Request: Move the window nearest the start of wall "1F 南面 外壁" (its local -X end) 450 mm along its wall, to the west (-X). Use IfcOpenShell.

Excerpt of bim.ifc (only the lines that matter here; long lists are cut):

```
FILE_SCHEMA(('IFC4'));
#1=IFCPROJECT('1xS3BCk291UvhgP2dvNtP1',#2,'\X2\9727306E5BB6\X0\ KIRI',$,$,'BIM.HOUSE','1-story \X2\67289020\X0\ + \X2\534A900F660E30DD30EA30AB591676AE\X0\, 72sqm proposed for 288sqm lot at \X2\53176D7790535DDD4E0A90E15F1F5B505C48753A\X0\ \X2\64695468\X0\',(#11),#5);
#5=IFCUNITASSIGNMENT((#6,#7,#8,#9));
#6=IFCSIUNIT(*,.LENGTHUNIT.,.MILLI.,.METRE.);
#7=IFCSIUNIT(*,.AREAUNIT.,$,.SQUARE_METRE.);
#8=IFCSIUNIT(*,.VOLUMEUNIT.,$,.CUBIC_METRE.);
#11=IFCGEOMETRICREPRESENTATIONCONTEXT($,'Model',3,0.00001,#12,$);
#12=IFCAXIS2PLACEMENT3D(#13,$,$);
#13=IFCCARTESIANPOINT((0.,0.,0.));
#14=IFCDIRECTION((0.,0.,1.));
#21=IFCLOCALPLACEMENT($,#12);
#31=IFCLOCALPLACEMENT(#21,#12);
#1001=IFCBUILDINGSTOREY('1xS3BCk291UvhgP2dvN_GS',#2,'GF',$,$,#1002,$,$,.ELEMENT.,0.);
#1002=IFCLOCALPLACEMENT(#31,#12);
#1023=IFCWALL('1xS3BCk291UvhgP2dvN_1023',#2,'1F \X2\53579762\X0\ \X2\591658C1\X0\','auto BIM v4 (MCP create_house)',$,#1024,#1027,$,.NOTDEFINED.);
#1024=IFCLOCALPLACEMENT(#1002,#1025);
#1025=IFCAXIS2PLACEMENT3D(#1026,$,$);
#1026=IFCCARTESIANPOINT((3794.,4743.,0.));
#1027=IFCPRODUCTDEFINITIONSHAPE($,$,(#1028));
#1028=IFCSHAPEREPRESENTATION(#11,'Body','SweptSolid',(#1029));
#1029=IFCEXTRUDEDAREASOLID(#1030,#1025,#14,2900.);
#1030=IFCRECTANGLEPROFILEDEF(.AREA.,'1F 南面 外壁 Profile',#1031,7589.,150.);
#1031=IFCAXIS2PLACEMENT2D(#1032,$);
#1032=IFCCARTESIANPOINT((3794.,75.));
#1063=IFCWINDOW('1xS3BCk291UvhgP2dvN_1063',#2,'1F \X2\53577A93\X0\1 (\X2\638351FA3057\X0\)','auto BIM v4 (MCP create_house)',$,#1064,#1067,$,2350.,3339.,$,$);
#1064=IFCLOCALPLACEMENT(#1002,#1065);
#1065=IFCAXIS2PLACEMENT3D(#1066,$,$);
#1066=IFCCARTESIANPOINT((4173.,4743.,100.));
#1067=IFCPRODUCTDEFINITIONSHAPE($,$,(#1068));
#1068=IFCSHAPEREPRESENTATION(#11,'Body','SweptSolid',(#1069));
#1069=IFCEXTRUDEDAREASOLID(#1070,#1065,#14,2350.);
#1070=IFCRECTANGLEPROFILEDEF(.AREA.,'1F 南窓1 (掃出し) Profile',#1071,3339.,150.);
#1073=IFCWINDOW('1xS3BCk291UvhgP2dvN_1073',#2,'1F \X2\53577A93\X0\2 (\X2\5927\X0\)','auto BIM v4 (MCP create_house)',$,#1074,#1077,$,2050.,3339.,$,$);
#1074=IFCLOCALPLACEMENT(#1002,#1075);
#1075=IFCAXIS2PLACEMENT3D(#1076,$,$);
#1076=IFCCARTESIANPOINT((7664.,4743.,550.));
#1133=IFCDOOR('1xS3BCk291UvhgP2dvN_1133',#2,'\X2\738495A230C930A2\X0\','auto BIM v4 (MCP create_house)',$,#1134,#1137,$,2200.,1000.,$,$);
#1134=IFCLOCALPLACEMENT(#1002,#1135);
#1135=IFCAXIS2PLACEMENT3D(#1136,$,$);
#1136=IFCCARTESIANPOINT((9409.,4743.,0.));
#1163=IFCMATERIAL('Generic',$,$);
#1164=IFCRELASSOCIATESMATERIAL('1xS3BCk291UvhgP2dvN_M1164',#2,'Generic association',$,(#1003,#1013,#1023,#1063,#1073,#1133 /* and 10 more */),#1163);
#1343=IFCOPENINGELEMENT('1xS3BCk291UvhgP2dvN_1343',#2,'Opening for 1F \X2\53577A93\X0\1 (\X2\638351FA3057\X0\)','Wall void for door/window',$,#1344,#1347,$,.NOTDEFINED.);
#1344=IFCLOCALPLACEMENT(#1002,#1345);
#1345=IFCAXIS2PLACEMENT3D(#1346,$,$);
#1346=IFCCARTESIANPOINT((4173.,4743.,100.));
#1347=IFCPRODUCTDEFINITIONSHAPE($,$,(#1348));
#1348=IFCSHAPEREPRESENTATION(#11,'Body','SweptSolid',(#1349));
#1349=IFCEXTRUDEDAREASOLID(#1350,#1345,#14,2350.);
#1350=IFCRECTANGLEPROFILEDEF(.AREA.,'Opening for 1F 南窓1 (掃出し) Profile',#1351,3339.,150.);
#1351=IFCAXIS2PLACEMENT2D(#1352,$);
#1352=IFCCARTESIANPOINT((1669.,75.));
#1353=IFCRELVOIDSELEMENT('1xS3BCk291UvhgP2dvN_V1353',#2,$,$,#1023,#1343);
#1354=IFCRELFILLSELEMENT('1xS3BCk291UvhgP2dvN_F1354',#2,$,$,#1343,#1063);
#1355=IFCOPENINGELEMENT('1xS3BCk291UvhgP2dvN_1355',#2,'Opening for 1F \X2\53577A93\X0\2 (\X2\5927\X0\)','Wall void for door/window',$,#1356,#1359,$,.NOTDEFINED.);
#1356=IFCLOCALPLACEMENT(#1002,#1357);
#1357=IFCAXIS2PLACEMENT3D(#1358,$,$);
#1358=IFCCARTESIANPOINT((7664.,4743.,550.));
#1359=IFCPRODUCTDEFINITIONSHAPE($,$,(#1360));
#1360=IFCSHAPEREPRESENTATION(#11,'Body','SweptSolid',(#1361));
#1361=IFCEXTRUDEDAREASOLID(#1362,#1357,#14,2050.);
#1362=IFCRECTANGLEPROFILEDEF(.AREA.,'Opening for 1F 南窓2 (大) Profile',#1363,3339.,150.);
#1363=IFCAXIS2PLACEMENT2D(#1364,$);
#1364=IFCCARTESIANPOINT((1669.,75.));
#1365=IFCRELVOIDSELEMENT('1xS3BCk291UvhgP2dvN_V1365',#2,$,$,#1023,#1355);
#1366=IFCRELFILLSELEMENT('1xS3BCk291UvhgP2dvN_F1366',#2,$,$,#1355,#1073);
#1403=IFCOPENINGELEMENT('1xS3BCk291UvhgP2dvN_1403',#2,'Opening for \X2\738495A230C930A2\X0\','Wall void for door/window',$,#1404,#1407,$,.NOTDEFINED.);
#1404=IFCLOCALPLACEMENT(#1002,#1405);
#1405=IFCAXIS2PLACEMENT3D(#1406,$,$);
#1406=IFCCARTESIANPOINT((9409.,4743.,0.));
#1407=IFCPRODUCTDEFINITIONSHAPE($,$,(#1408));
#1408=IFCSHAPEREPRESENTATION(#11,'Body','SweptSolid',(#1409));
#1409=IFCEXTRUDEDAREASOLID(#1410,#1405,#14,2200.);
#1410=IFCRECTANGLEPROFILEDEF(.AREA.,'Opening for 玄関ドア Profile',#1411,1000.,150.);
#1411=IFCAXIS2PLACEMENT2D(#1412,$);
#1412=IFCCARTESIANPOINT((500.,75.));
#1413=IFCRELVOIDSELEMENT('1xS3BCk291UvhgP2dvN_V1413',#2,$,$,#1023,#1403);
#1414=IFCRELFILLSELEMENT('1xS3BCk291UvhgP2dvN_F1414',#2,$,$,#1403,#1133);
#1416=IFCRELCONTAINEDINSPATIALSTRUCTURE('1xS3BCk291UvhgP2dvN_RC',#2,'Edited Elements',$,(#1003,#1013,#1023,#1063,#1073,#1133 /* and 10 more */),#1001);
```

```python
import ifcopenshell
import ifcopenshell.api.geometry
import ifcopenshell.util.placement

model = ifcopenshell.open("bim.ifc")

window = model.by_guid("1xS3BCk291UvhgP2dvN_1063")
opening = window.FillsVoids[0].RelatingOpeningElement
wall = opening.VoidsElements[0].RelatingBuildingElement

wall_matrix = ifcopenshell.util.placement.get_local_placement(wall.ObjectPlacement)
shift = wall_matrix[:3, 0] * -450.0
before = ifcopenshell.util.placement.get_local_placement(window.ObjectPlacement)[:3, 3].copy()

# The window is not placed relative to its opening, so move both.
for product in (opening, window):
    matrix = ifcopenshell.util.placement.get_local_placement(product.ObjectPlacement)
    matrix[:3, 3] += shift
    ifcopenshell.api.geometry.edit_object_placement(model, product=product, matrix=matrix, is_si=False)

after = ifcopenshell.util.placement.get_local_placement(window.ObjectPlacement)[:3, 3]
print("window moved by", (after - before).round(3) + 0.0)

model.write("bim-out.ifc")
```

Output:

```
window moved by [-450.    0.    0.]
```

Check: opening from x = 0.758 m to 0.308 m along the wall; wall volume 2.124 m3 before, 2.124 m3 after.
